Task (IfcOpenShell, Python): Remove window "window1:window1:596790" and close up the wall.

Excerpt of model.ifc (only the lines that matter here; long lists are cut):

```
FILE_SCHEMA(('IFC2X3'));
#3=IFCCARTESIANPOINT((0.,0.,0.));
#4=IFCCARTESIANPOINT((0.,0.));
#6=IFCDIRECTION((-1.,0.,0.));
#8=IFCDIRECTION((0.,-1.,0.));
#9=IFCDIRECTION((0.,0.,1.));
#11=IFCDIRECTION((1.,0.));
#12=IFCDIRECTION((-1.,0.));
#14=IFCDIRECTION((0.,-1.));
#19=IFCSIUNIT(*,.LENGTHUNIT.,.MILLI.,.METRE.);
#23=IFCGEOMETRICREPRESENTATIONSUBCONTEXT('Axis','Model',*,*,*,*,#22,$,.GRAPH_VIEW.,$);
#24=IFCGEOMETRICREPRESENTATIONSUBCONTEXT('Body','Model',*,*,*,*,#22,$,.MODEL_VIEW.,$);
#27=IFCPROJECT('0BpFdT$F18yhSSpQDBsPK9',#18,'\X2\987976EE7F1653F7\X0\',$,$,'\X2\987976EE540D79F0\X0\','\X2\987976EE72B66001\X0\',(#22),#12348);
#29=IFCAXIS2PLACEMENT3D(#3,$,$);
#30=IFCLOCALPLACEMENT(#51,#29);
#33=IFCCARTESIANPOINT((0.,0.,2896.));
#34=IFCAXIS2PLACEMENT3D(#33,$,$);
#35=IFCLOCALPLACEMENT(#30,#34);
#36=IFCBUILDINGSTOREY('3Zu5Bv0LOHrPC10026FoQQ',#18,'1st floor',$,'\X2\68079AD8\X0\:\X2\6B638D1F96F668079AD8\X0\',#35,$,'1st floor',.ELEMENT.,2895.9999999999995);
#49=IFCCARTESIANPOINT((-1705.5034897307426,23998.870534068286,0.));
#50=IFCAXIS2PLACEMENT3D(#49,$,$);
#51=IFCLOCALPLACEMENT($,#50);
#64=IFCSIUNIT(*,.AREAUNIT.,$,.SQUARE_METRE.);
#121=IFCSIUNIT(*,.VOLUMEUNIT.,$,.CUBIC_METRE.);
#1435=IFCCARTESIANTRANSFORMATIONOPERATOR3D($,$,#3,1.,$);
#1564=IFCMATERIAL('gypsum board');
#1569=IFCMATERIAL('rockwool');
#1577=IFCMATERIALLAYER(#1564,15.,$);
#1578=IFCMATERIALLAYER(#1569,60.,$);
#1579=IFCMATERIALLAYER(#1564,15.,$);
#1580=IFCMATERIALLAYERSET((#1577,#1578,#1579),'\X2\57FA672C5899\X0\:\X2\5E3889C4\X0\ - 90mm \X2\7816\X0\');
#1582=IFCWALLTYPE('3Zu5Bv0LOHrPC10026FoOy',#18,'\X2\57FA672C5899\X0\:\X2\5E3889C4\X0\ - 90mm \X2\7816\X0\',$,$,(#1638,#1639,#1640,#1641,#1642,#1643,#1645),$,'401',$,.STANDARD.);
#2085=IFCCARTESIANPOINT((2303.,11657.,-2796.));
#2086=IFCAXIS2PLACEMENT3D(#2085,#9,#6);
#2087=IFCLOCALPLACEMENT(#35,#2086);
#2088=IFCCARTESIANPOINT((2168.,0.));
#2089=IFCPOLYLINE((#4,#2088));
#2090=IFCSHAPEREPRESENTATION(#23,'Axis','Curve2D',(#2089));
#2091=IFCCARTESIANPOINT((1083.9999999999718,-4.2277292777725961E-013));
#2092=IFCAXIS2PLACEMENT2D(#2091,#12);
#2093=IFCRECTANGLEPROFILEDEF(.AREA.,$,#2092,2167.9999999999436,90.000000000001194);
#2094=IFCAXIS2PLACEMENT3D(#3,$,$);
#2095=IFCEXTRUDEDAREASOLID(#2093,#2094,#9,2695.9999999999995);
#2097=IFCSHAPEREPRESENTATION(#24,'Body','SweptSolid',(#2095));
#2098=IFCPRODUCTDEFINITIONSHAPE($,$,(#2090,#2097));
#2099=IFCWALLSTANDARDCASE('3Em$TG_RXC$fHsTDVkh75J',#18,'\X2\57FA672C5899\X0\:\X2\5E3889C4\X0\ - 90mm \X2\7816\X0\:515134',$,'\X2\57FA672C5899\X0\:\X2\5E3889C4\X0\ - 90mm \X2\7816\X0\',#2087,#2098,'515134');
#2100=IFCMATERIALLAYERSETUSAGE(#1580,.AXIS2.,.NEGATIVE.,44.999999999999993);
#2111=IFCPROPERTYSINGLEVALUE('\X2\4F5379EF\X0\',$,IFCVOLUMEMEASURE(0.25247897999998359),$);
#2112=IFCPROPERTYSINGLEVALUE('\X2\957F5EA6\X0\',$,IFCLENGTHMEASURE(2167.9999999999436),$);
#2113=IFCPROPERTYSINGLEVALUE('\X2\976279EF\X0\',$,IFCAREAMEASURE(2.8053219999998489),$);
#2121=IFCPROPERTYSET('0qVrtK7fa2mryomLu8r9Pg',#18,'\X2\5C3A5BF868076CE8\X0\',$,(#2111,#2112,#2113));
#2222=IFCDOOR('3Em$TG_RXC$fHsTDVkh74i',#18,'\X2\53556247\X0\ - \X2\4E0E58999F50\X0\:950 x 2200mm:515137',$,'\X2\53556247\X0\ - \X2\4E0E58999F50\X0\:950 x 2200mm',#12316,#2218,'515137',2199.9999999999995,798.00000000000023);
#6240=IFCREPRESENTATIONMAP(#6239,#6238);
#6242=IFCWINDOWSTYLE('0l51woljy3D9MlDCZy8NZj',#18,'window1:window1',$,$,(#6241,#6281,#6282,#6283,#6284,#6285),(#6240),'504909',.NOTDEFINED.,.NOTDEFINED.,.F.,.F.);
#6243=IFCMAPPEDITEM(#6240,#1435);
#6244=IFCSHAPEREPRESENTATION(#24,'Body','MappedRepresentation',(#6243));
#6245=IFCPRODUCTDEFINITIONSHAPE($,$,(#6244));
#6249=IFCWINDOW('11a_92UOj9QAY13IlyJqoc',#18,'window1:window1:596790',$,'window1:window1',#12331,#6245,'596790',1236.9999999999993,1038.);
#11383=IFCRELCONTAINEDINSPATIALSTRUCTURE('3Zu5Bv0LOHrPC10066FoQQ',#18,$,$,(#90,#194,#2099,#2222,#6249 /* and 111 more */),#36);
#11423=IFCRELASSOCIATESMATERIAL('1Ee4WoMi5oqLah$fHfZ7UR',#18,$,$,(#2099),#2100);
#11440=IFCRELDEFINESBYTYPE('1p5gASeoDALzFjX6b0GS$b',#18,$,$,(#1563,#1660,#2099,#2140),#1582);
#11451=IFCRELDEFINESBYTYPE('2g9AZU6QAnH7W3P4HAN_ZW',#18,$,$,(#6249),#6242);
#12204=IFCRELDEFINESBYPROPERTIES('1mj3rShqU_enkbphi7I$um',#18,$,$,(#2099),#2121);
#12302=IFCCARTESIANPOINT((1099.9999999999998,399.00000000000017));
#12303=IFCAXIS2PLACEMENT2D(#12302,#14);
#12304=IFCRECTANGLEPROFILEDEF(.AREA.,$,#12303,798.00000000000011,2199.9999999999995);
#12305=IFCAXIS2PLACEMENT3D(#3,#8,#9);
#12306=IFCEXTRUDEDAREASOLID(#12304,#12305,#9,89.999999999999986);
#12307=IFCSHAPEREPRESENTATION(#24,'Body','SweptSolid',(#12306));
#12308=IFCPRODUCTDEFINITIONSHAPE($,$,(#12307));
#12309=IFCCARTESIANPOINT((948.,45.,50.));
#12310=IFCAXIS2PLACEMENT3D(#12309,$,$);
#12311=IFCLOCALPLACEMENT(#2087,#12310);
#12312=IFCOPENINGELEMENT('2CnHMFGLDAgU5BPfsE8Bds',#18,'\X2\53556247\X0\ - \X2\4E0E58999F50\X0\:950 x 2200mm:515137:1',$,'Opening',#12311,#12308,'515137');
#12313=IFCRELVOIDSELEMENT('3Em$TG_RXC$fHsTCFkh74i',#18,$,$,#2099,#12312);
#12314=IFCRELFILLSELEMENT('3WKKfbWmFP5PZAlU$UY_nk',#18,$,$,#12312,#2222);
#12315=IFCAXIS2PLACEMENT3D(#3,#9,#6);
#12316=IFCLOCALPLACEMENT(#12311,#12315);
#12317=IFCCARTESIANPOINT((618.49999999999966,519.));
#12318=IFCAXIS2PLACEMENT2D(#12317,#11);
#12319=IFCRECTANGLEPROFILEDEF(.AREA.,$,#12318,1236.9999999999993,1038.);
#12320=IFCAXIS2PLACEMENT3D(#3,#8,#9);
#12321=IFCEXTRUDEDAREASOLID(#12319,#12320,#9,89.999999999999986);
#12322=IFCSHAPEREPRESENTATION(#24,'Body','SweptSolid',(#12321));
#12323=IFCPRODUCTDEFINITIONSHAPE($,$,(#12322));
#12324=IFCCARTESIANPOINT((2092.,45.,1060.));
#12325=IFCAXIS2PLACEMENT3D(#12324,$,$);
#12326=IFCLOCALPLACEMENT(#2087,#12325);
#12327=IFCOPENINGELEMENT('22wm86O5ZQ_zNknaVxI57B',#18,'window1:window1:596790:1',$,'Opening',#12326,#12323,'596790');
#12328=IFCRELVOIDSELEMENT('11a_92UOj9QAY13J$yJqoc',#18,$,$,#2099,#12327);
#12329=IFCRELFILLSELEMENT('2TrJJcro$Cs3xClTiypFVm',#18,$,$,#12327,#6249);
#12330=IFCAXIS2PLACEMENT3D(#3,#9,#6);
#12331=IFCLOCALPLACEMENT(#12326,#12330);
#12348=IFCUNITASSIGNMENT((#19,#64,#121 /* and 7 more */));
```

```python
import ifcopenshell
import ifcopenshell.api.feature
import ifcopenshell.api.pset
import ifcopenshell.api.root
import ifcopenshell.geom
import ifcopenshell.util.element
import ifcopenshell.util.shape
import ifcopenshell.util.unit

model = ifcopenshell.open("model.ifc")
area_scale = ifcopenshell.util.unit.calculate_unit_scale(model, "AREAUNIT")
volume_scale = ifcopenshell.util.unit.calculate_unit_scale(model, "VOLUMEUNIT")
settings = ifcopenshell.geom.settings()


def volume(element):
    """Net volume in cubic metres, openings subtracted."""
    shape = ifcopenshell.geom.create_shape(settings, element)
    return ifcopenshell.util.shape.get_volume(shape.geometry)


window = model.by_guid("11a_92UOj9QAY13IlyJqoc")
opening = window.FillsVoids[0].RelatingOpeningElement
wall = opening.VoidsElements[0].RelatingBuildingElement
before = volume(wall)

ifcopenshell.api.root.remove_product(model, product=window)
ifcopenshell.api.feature.remove_feature(model, feature=opening)

after = volume(wall)
thickness = 0.09  # wall thickness in metres

# Update the wall's stored quantities.
pset = model.by_id(ifcopenshell.util.element.get_pset(wall, "尺寸标注", should_inherit=False)["id"])
ifcopenshell.api.pset.edit_pset(model, pset=pset, properties={
    "体积": model.create_entity("IfcVolumeMeasure", after / volume_scale),
    "面积": model.create_entity("IfcAreaMeasure", after / thickness / area_scale),
})

print(f"wall volume {before:.3f} -> {after:.3f} m3")

model.write("model-out.ifc")
```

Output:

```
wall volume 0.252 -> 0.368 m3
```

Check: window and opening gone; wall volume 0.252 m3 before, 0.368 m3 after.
